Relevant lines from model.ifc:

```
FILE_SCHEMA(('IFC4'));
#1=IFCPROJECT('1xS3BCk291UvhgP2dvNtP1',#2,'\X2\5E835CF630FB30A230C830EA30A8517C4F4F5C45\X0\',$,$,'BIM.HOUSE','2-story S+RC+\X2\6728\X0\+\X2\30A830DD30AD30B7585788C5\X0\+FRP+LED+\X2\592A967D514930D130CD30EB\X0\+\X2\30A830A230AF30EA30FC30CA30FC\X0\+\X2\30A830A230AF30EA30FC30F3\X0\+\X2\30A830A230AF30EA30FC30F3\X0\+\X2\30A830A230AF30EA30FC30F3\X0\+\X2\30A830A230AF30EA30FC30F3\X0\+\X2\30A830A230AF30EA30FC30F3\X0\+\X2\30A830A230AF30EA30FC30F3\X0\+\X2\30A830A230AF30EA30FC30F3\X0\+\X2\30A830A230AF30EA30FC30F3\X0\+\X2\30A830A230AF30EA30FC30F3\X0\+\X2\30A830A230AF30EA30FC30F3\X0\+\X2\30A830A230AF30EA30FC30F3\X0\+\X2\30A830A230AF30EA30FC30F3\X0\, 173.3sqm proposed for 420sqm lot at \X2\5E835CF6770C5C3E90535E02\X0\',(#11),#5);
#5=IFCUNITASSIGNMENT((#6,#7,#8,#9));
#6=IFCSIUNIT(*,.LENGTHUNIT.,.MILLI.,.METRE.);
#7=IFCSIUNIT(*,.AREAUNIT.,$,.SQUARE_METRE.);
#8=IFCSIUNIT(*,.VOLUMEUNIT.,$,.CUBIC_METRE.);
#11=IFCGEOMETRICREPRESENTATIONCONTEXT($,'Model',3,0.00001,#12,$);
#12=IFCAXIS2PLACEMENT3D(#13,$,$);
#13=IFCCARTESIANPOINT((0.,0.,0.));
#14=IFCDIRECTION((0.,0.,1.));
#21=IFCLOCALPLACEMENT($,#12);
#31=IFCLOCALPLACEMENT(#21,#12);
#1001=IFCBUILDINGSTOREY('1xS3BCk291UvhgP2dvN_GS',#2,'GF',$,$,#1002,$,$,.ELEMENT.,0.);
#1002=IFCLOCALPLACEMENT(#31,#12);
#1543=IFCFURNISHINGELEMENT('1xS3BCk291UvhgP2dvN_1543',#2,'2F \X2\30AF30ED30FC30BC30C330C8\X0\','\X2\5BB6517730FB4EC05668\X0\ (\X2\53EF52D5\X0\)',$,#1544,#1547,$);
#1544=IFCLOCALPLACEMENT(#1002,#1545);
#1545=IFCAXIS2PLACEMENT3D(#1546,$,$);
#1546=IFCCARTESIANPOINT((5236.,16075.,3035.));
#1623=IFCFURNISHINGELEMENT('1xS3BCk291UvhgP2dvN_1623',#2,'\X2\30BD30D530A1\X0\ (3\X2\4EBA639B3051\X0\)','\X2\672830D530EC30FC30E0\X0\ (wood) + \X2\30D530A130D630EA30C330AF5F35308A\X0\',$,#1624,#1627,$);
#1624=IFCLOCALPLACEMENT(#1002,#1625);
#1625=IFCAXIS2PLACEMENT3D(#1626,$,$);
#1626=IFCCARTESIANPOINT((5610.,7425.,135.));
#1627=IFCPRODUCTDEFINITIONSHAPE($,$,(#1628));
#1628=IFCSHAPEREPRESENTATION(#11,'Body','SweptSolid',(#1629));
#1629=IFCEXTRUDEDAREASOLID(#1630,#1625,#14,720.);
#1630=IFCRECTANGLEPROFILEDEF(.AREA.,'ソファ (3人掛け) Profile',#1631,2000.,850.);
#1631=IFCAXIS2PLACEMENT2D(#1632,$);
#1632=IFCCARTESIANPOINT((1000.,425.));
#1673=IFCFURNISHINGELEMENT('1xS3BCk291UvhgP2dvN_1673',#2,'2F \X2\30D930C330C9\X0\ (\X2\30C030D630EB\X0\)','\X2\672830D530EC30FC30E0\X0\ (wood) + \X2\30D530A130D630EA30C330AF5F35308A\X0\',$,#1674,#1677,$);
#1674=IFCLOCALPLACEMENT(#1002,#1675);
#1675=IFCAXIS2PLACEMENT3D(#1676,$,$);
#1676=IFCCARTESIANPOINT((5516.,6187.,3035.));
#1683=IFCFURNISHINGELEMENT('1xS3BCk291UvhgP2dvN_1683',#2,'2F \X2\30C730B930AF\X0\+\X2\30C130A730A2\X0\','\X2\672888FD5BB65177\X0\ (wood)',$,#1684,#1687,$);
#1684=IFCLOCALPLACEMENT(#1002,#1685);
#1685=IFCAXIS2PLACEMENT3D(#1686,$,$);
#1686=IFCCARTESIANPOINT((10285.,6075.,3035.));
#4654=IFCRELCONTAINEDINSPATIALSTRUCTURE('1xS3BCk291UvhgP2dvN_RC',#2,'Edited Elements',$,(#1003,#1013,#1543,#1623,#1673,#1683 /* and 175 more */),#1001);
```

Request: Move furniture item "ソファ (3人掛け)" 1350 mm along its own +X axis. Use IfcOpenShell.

```python
import ifcopenshell
import ifcopenshell.api.geometry
import ifcopenshell.util.placement
import ifcopenshell.util.unit

model = ifcopenshell.open("model.ifc")
unit_scale = ifcopenshell.util.unit.calculate_unit_scale(model)

item = model.by_guid("1xS3BCk291UvhgP2dvN_1623")
matrix = ifcopenshell.util.placement.get_local_placement(item.ObjectPlacement)
matrix[:3, 3] += matrix[:3, 0] * 1.35 / unit_scale
ifcopenshell.api.geometry.edit_object_placement(model, product=item, matrix=matrix, is_si=False)

print(ifcopenshell.util.placement.get_local_placement(item.ObjectPlacement).round(3) + 0.0)

model.write("model-out.ifc")
```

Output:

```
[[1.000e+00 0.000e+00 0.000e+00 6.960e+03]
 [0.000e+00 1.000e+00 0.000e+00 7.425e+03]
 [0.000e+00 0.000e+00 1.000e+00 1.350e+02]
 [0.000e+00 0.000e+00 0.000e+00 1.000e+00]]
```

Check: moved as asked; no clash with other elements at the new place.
